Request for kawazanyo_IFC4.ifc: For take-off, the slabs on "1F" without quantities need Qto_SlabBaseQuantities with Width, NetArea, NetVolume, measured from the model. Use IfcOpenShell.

First a look at what the model holds.

```python
import ifcopenshell
import ifcopenshell.util.element
import ifcopenshell.util.unit

model = ifcopenshell.open("kawazanyo_IFC4.ifc")
print(model.schema)
for unit_type in ("LENGTHUNIT", "AREAUNIT", "VOLUMEUNIT"):
    print(unit_type, ifcopenshell.util.unit.calculate_unit_scale(model, unit_type))
storey = next(s for s in model.by_type("IfcBuildingStorey") if s.Name == "1F")
slabs = [e for e in ifcopenshell.util.element.get_decomposition(storey) if e.is_a("IfcSlab")]
for e in sorted(slabs, key=lambda e: e.id()):
    print(e.id(), e.is_a(), e.Name, list(ifcopenshell.util.element.get_psets(e, qtos_only=True)), sep=" | ")
```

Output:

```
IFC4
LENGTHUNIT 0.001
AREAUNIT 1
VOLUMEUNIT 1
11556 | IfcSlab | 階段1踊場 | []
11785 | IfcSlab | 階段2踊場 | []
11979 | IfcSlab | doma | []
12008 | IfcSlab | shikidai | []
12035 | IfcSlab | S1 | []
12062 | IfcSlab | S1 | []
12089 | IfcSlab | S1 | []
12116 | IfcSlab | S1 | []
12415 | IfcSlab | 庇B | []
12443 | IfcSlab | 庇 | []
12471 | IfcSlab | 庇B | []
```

```python
import ifcopenshell
import ifcopenshell.api.pset
import ifcopenshell.geom
import ifcopenshell.util.element
import ifcopenshell.util.shape
import ifcopenshell.util.unit

model = ifcopenshell.open("kawazanyo_IFC4.ifc")
unit_scale = ifcopenshell.util.unit.calculate_unit_scale(model)
area_scale = ifcopenshell.util.unit.calculate_unit_scale(model, "AREAUNIT")
volume_scale = ifcopenshell.util.unit.calculate_unit_scale(model, "VOLUMEUNIT")
settings = ifcopenshell.geom.settings()

storey = next(s for s in model.by_type("IfcBuildingStorey") if s.Name == "1F")
slabs = [e for e in ifcopenshell.util.element.get_decomposition(storey) if e.is_a("IfcSlab")]

for e in sorted(slabs, key=lambda e: e.id()):
    if ifcopenshell.util.element.get_psets(e, qtos_only=True, should_inherit=False):
        continue
    # Geometry comes back in metres, in the element's own axes.
    shape = ifcopenshell.geom.create_shape(settings, e)
    values = {
        "Width": ifcopenshell.util.shape.get_z(shape.geometry) / unit_scale,
        "NetArea": ifcopenshell.util.shape.get_footprint_area(shape.geometry) / area_scale,
        "NetVolume": ifcopenshell.util.shape.get_volume(shape.geometry) / volume_scale,
    }
    qto = ifcopenshell.api.pset.add_qto(model, product=e, name="Qto_SlabBaseQuantities")
    ifcopenshell.api.pset.edit_qto(model, qto=qto, properties=values)
    print(e.id(), {k: round(v, 3) for k, v in values.items()})

model.write("kawazanyo_IFC4_v2.ifc")
```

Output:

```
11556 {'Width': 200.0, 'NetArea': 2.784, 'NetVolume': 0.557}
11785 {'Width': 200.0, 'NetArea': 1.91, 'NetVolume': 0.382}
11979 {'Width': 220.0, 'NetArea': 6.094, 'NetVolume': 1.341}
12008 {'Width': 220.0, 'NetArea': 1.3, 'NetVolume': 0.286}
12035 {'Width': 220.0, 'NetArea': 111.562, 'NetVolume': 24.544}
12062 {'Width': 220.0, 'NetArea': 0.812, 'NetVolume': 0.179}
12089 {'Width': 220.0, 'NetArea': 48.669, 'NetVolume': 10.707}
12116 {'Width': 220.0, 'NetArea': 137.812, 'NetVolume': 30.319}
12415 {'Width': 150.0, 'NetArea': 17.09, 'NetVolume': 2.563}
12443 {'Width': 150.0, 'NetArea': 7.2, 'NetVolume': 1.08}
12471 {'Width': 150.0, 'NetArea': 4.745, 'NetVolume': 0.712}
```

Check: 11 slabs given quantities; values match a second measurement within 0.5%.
